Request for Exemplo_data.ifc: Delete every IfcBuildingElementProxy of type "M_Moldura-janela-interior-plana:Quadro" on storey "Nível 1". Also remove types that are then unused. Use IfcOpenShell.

First a look at what the model holds.

```python
import ifcopenshell
import ifcopenshell.util.element

model = ifcopenshell.open("Exemplo_data.ifc")
print(model.schema)
storey = next(s for s in model.by_type("IfcBuildingStorey") if s.Name == "Nível 1")
proxies = [e for e in ifcopenshell.util.element.get_decomposition(storey) if e.is_a("IfcBuildingElementProxy")]
seen = {}
for e in proxies:
    element_type = ifcopenshell.util.element.get_type(e)
    name = element_type.Name if element_type not in (None, e) else None
    seen[name] = seen.get(name, 0) + 1
for name, count in sorted(seen.items(), key=str):
    print(count, "x", name)
```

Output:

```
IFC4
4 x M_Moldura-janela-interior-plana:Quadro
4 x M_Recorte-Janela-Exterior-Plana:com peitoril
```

```python
import ifcopenshell
import ifcopenshell.api.root
import ifcopenshell.util.element

model = ifcopenshell.open("Exemplo_data.ifc")

storey = next(s for s in model.by_type("IfcBuildingStorey") if s.Name == "Nível 1")
proxies = [e for e in ifcopenshell.util.element.get_decomposition(storey) if e.is_a("IfcBuildingElementProxy")]
targets = [e for e in proxies if (t := ifcopenshell.util.element.get_type(e)) not in (None, e) and t.Name == "M_Moldura-janela-interior-plana:Quadro"]
types = {ifcopenshell.util.element.get_type(e) for e in targets} - {None, *targets}

for e in targets:
    ifcopenshell.api.root.remove_product(model, product=e)
print(len(targets), "removed")

unused = [t for t in types if not ifcopenshell.util.element.get_types(t)]
for t in unused:
    ifcopenshell.api.root.remove_product(model, product=t)
print(len(unused), "unused types removed")

model.write("Exemplo_data-out.ifc")
```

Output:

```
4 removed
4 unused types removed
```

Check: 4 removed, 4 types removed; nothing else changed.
